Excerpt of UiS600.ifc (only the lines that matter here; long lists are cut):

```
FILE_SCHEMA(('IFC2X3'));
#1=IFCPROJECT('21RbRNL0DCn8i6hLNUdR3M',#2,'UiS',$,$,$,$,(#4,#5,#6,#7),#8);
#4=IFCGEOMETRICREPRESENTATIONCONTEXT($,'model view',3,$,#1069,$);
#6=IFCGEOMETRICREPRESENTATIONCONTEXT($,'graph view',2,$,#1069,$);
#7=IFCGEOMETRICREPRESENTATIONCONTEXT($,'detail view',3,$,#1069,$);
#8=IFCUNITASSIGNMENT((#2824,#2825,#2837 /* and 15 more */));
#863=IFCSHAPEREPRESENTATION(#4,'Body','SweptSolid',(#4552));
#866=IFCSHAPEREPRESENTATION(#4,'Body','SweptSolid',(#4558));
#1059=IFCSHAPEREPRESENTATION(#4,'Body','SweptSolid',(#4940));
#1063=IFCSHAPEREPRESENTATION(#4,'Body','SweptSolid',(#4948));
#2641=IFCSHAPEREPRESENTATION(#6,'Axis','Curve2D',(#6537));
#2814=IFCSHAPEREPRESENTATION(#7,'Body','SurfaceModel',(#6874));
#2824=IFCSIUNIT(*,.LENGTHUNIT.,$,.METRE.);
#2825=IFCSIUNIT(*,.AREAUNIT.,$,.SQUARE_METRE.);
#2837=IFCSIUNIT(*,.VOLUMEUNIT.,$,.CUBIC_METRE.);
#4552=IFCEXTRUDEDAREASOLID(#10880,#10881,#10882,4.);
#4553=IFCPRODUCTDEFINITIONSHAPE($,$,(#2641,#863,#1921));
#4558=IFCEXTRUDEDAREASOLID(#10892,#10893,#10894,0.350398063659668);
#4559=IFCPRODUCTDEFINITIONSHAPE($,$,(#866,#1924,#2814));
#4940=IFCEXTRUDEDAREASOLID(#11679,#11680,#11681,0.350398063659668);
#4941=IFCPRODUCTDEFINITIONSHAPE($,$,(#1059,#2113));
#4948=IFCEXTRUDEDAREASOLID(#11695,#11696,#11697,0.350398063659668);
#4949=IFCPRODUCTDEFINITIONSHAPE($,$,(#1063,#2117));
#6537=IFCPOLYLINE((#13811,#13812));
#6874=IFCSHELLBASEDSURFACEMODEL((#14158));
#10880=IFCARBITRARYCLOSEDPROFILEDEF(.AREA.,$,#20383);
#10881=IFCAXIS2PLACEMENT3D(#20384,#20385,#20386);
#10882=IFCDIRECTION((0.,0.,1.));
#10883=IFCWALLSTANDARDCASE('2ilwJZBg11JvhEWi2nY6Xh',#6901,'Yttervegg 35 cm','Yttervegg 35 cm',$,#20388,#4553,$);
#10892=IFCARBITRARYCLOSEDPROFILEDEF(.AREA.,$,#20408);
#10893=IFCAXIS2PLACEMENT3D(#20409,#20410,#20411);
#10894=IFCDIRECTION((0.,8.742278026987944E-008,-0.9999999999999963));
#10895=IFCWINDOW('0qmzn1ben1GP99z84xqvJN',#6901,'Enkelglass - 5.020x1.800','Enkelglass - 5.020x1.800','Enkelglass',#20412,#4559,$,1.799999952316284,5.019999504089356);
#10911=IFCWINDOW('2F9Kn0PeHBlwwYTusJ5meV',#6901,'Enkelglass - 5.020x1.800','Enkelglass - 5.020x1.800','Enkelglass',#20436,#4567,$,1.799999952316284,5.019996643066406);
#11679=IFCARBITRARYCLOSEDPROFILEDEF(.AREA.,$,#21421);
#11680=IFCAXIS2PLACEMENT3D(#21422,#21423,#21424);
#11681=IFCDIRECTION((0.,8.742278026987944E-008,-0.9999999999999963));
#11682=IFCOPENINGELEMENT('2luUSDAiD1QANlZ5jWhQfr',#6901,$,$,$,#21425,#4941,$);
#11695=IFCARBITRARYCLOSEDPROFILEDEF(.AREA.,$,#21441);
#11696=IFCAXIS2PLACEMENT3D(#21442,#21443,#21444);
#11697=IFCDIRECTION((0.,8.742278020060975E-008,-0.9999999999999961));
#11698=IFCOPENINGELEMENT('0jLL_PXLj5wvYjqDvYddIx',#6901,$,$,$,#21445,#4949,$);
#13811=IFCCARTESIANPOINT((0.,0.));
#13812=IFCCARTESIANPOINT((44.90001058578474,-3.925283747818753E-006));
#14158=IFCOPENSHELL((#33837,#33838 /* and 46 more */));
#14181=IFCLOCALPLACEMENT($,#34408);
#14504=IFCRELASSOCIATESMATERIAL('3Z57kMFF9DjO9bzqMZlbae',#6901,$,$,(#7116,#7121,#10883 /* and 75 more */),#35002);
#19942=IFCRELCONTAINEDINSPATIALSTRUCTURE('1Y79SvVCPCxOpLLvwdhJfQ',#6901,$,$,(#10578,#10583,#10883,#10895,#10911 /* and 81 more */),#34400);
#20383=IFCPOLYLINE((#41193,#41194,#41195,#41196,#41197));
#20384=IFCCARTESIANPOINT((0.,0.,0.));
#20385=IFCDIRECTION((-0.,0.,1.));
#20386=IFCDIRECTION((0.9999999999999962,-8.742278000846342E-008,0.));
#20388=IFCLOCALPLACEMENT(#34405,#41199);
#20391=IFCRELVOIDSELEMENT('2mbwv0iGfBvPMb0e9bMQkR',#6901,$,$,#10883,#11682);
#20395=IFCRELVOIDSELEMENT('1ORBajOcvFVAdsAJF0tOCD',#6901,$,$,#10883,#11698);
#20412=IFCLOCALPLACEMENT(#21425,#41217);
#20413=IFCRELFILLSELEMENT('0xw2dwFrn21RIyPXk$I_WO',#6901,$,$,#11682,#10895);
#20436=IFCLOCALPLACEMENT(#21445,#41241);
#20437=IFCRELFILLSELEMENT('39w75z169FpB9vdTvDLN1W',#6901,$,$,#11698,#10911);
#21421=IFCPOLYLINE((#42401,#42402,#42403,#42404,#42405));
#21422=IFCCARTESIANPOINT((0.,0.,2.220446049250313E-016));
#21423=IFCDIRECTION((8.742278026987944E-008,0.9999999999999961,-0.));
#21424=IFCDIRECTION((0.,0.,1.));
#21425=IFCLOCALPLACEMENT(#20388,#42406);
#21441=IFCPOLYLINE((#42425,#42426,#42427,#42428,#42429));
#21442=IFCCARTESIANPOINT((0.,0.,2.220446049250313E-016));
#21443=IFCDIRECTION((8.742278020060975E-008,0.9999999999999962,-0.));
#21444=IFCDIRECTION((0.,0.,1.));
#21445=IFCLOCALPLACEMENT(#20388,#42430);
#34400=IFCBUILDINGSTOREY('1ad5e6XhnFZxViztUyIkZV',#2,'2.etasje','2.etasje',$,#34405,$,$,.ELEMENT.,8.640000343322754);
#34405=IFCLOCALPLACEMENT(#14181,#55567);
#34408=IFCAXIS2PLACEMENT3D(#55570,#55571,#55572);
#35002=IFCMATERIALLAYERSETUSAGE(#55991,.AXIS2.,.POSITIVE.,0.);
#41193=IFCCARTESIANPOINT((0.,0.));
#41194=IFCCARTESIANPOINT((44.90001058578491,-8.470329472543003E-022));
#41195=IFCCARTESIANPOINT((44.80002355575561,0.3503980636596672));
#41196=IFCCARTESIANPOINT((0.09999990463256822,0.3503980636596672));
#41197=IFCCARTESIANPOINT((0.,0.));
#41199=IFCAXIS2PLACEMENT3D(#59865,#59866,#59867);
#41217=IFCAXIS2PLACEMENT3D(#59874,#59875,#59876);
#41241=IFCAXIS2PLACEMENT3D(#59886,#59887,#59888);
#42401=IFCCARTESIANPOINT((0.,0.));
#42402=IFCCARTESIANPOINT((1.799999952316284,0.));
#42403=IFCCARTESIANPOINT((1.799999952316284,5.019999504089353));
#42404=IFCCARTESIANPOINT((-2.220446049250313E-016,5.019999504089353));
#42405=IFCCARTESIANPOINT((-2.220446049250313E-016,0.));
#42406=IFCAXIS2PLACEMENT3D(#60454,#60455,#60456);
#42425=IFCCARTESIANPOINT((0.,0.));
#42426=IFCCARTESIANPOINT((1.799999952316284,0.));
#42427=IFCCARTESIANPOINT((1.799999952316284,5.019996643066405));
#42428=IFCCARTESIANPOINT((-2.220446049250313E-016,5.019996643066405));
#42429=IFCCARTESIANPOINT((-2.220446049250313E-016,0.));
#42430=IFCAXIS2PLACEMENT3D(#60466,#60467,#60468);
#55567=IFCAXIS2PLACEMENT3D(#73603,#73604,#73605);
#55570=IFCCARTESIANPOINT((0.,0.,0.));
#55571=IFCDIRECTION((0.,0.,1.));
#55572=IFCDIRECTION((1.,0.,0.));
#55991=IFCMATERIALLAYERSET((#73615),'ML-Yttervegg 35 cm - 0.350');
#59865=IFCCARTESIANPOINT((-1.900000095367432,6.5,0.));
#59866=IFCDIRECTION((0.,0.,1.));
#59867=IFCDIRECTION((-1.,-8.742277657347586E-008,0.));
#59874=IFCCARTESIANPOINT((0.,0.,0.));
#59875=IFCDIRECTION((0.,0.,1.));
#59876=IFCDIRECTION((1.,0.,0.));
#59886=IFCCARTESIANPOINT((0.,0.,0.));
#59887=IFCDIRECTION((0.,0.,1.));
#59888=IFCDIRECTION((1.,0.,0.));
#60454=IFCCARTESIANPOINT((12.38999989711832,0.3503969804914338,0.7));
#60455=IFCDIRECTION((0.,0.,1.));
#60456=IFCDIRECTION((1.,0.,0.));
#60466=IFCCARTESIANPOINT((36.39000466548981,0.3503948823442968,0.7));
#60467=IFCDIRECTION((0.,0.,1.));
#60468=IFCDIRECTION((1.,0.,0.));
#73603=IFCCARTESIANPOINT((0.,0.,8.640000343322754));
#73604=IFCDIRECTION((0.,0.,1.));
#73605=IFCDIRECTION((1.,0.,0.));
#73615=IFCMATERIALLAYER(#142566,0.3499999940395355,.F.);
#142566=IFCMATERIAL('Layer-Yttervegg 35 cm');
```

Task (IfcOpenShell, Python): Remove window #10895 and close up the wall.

```python
import ifcopenshell
import ifcopenshell.api.feature
import ifcopenshell.api.root
import ifcopenshell.geom
import ifcopenshell.util.shape

model = ifcopenshell.open("UiS600.ifc")
settings = ifcopenshell.geom.settings()


def volume(element):
    """Net volume in cubic metres, openings subtracted."""
    shape = ifcopenshell.geom.create_shape(settings, element)
    return ifcopenshell.util.shape.get_volume(shape.geometry)


window = model.by_guid("0qmzn1ben1GP99z84xqvJN")
opening = window.FillsVoids[0].RelatingOpeningElement
wall = opening.VoidsElements[0].RelatingBuildingElement
before = volume(wall)

ifcopenshell.api.root.remove_product(model, product=window)
ifcopenshell.api.feature.remove_feature(model, feature=opening)

after = volume(wall)

print(f"wall volume {before:.3f} -> {after:.3f} m3")

model.write("UiS600-out.ifc")
```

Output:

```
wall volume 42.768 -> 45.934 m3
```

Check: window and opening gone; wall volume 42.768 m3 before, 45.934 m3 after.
